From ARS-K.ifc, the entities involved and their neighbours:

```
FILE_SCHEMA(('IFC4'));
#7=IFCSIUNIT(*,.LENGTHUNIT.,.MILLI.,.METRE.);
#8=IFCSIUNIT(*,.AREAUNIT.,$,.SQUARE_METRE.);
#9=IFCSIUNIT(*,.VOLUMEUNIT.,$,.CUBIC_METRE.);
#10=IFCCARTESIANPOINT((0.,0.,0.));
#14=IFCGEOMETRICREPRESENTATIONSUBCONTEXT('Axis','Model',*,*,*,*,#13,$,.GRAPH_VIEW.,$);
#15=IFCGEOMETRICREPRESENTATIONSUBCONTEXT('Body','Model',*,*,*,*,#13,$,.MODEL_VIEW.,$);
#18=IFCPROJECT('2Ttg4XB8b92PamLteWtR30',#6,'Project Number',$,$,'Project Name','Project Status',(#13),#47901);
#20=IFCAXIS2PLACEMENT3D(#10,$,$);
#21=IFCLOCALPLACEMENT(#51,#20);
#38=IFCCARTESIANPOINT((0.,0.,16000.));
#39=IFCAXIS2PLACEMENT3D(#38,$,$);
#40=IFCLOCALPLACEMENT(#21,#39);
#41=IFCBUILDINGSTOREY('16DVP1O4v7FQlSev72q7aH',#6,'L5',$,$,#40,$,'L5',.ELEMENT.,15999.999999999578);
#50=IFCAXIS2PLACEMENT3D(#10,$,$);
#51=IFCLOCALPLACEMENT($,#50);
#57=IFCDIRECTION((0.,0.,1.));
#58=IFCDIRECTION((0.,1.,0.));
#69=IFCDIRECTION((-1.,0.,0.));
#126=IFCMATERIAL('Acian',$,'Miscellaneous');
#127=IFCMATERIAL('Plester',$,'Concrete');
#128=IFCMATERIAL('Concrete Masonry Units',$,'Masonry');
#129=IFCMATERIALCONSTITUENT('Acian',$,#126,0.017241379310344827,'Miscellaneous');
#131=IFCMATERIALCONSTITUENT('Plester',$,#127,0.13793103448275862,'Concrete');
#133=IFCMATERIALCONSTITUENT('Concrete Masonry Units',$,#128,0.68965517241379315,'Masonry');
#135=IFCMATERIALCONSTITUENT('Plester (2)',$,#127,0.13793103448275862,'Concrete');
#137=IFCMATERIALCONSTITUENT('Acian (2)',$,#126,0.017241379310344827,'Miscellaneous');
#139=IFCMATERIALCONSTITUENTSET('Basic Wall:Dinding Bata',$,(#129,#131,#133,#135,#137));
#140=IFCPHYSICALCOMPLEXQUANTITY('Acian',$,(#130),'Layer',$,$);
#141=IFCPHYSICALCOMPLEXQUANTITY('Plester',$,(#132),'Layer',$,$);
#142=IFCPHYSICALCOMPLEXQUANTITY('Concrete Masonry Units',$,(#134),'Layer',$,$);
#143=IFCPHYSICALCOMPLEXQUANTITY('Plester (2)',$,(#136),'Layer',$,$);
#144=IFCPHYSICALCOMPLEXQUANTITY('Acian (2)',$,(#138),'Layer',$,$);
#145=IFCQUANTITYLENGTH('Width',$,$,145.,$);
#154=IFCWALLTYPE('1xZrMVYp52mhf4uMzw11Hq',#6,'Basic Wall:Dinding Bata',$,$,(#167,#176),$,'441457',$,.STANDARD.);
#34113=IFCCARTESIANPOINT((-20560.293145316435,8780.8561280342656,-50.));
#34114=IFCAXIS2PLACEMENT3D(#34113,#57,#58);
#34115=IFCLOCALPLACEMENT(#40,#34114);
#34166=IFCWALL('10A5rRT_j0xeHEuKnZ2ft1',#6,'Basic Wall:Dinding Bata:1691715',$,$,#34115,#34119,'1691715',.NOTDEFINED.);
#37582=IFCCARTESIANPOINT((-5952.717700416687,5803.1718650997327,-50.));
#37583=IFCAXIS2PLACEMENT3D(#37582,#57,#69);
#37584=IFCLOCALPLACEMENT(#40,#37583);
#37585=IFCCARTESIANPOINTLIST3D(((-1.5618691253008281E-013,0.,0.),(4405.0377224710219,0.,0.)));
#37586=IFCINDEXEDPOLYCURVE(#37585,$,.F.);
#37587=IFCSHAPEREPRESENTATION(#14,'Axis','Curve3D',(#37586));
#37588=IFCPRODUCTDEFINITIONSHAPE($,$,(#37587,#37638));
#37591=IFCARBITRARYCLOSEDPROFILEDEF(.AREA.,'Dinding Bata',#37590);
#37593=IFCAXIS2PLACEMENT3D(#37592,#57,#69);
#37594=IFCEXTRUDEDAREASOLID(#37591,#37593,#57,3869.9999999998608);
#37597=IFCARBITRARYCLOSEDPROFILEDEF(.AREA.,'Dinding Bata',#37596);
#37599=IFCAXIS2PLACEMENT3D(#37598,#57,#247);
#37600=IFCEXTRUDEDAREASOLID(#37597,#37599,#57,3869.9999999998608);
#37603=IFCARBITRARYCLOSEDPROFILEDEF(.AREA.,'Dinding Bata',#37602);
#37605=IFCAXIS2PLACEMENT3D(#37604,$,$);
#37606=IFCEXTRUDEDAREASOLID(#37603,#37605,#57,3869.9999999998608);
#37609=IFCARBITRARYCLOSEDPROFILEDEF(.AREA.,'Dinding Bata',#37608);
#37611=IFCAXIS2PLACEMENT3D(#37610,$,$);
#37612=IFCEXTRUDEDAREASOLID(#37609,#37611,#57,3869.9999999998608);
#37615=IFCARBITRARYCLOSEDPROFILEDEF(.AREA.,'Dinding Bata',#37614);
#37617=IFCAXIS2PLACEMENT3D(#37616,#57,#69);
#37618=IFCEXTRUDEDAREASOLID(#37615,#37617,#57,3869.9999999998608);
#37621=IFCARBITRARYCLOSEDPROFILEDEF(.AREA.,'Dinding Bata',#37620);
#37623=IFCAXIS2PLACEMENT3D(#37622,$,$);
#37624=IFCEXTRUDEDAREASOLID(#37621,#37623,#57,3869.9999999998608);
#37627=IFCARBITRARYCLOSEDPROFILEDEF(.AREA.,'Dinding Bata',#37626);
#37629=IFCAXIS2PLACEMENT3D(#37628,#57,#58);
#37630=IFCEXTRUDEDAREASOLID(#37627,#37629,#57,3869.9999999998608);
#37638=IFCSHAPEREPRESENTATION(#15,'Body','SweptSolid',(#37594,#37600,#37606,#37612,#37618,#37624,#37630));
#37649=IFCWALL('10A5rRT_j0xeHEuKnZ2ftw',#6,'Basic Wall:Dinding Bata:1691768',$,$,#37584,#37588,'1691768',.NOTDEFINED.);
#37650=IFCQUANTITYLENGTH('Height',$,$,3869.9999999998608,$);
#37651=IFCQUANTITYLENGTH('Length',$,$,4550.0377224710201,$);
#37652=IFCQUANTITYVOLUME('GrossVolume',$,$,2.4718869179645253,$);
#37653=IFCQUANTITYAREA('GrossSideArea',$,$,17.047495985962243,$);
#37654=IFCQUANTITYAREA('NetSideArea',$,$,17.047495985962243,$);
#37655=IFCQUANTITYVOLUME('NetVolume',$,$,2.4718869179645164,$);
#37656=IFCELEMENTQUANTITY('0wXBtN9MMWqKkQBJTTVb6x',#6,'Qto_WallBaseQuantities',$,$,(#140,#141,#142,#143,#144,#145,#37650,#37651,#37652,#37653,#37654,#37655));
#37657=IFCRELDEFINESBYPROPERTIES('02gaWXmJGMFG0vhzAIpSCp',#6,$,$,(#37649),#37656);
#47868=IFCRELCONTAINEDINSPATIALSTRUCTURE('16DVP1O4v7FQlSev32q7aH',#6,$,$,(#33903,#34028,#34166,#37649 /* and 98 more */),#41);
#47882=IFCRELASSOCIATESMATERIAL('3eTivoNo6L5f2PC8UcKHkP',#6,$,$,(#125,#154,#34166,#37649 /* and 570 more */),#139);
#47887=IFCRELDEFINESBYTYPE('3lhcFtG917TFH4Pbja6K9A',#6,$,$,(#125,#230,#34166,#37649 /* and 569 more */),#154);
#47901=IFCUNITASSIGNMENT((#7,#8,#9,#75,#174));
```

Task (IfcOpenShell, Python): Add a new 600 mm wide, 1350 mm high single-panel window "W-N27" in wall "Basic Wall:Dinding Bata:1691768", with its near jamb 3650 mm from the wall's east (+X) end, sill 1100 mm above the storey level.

```python
import numpy as np
import ifcopenshell
import ifcopenshell.api.feature
import ifcopenshell.api.geometry
import ifcopenshell.api.pset
import ifcopenshell.api.root
import ifcopenshell.api.spatial
import ifcopenshell.geom
import ifcopenshell.util.element
import ifcopenshell.util.placement
import ifcopenshell.util.representation
import ifcopenshell.util.shape
import ifcopenshell.util.unit

model = ifcopenshell.open("ARS-K.ifc")
unit_scale = ifcopenshell.util.unit.calculate_unit_scale(model)
area_scale = ifcopenshell.util.unit.calculate_unit_scale(model, "AREAUNIT")
volume_scale = ifcopenshell.util.unit.calculate_unit_scale(model, "VOLUMEUNIT")
settings = ifcopenshell.geom.settings()


def volume(element):
    """Net volume in cubic metres, openings subtracted."""
    shape = ifcopenshell.geom.create_shape(settings, element)
    return ifcopenshell.util.shape.get_volume(shape.geometry)


wall = model.by_guid("10A5rRT_j0xeHEuKnZ2ftw")
storey = ifcopenshell.util.element.get_container(wall, ifc_class="IfcBuildingStorey")
context = ifcopenshell.util.representation.get_context(model, "Model", "Body", "MODEL_VIEW")
before = volume(wall)

width, height, from_end, sill = 0.6, 1.35, 3.65, 1.1  # metres

# The wall runs along its own X axis, and the end named is its -X end.
wall_shape = ifcopenshell.geom.create_shape(settings, wall)
x, y, z = ifcopenshell.util.shape.get_vertices(wall_shape.geometry).T
start = x.min() + from_end
face, thickness = float(y.min()), float(y.max() - y.min())
wall_matrix = ifcopenshell.util.placement.get_local_placement(wall.ObjectPlacement)
level = ifcopenshell.util.placement.get_local_placement(storey.ObjectPlacement)[2, 3]


def in_wall(x, y):
    """Placement at x, y metres in the wall's axes, at sill height."""
    matrix = wall_matrix.copy()
    matrix[:, 3] = wall_matrix @ np.array([x / unit_scale, y / unit_scale, 0.0, 1.0])
    matrix[2, 3] = level + sill / unit_scale
    return matrix


# Opening: a box that overshoots both wall faces by 50 mm.
opening = ifcopenshell.api.root.create_entity(model, ifc_class="IfcOpeningElement", predefined_type="OPENING")
box = ifcopenshell.api.geometry.add_wall_representation(
    model, context=context, length=width, height=height, thickness=thickness + 0.1
)
ifcopenshell.api.geometry.assign_representation(model, product=opening, representation=box)
ifcopenshell.api.geometry.edit_object_placement(model, product=opening, matrix=in_wall(start, face - 0.05), is_si=False)
ifcopenshell.api.feature.add_feature(model, feature=opening, element=wall)

window = ifcopenshell.api.root.create_entity(model, ifc_class="IfcWindow", name="W-N27", predefined_type="WINDOW")
window.OverallWidth, window.OverallHeight = width / unit_scale, height / unit_scale
window.PartitioningType = "SINGLE_PANEL"
body = ifcopenshell.api.geometry.add_window_representation(
    model,
    context=context,
    overall_width=window.OverallWidth,
    overall_height=window.OverallHeight,
    partition_type="SINGLE_PANEL",
)
ifcopenshell.api.geometry.assign_representation(model, product=window, representation=body)
ifcopenshell.api.spatial.assign_container(model, products=[window], relating_structure=storey)
ifcopenshell.api.feature.add_filling(model, opening=opening, element=window)

# Centre the window in the wall's thickness.
ifcopenshell.api.geometry.edit_object_placement(model, product=window, matrix=in_wall(start, face), is_si=False)
window_shape = ifcopenshell.geom.create_shape(settings, window)
depth = ifcopenshell.util.shape.get_vertices(window_shape.geometry)[:, 1]
offset = face + thickness / 2 - (depth.min() + depth.max()) / 2
ifcopenshell.api.geometry.edit_object_placement(model, product=window, matrix=in_wall(start, offset), is_si=False)

after = volume(wall)

# Update the wall's stored quantities.
qto = model.by_id(ifcopenshell.util.element.get_pset(wall, "Qto_WallBaseQuantities", should_inherit=False)["id"])
ifcopenshell.api.pset.edit_qto(model, qto=qto, properties={
    "NetSideArea": after / thickness / area_scale,
    "NetVolume": after / volume_scale,
})

print(f"wall volume {before:.3f} -> {after:.3f} m3")

model.write("ARS-K-out.ifc")
```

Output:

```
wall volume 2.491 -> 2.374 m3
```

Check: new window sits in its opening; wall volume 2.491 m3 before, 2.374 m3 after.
